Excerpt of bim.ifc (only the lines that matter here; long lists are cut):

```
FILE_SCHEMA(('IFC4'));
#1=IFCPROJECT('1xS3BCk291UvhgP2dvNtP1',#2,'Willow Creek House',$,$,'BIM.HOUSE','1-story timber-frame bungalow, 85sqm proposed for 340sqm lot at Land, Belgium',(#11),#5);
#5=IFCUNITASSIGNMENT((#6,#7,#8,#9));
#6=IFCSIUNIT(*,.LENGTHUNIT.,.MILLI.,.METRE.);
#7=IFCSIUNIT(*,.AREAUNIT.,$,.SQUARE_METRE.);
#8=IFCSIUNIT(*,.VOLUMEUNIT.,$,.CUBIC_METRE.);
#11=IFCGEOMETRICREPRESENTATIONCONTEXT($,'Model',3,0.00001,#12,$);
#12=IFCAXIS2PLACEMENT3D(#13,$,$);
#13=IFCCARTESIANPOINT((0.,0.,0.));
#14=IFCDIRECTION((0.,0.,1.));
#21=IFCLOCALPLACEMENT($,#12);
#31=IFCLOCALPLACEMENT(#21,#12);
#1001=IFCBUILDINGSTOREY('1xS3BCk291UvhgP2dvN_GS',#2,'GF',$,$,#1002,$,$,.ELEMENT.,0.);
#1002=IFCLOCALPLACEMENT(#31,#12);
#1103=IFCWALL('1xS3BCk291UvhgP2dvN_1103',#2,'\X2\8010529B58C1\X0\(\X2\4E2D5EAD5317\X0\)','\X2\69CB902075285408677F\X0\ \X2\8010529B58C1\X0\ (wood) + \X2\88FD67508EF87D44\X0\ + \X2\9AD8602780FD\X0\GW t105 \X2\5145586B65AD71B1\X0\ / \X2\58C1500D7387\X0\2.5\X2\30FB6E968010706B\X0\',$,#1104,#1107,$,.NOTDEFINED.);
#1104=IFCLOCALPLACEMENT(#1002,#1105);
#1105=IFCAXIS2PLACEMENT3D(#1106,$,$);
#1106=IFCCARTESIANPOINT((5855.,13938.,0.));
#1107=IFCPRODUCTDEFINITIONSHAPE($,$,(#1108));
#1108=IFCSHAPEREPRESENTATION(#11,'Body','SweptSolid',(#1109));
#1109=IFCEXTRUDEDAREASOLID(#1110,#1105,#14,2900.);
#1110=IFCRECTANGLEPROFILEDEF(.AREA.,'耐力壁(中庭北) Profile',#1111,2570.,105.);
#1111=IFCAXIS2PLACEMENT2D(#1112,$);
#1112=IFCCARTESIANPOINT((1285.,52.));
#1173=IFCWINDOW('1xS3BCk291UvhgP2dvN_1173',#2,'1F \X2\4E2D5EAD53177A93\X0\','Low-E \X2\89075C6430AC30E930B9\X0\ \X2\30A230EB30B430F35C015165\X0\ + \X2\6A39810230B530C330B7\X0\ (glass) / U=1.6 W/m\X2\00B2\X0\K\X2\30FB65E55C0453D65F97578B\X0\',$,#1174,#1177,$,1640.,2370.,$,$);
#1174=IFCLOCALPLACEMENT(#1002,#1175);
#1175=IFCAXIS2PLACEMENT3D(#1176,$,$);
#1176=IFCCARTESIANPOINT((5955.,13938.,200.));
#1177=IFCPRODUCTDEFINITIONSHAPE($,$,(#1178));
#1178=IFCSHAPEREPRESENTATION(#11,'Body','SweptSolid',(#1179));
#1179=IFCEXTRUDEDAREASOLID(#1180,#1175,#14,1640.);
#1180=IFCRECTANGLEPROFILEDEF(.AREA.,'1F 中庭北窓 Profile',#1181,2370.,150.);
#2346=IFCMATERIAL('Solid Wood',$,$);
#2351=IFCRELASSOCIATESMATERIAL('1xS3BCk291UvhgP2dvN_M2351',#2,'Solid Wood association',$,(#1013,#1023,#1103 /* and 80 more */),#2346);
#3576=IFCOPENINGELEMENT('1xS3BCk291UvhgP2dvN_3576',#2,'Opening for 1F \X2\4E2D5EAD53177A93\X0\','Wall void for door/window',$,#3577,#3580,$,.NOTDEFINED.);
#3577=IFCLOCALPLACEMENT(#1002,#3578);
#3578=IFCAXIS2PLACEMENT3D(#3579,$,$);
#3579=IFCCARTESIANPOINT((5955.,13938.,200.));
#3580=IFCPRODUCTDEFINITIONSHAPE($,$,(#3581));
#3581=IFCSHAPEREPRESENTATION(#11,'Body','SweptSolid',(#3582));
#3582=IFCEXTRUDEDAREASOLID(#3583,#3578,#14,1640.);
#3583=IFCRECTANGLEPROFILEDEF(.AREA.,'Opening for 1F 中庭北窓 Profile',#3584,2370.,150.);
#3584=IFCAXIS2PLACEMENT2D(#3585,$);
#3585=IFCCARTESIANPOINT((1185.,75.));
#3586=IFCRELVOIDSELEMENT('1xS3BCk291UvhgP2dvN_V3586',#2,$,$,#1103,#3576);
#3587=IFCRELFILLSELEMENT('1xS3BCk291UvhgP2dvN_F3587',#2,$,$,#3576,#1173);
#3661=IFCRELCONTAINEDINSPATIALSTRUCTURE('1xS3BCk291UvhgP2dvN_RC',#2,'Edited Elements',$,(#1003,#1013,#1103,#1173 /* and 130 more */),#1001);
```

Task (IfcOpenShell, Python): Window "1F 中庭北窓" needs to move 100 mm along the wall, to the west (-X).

```python
import ifcopenshell
import ifcopenshell.api.geometry
import ifcopenshell.util.placement

model = ifcopenshell.open("bim.ifc")

window = model.by_id(1173)
opening = window.FillsVoids[0].RelatingOpeningElement
wall = opening.VoidsElements[0].RelatingBuildingElement

wall_matrix = ifcopenshell.util.placement.get_local_placement(wall.ObjectPlacement)
shift = wall_matrix[:3, 0] * -100.0
before = ifcopenshell.util.placement.get_local_placement(window.ObjectPlacement)[:3, 3].copy()

# The window is not placed relative to its opening, so move both.
for product in (opening, window):
    matrix = ifcopenshell.util.placement.get_local_placement(product.ObjectPlacement)
    matrix[:3, 3] += shift
    ifcopenshell.api.geometry.edit_object_placement(model, product=product, matrix=matrix, is_si=False)

after = ifcopenshell.util.placement.get_local_placement(window.ObjectPlacement)[:3, 3]
print("window moved by", (after - before).round(3) + 0.0)

model.write("bim_updated.ifc")
```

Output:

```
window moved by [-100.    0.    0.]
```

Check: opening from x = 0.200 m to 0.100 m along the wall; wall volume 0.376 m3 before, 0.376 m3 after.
